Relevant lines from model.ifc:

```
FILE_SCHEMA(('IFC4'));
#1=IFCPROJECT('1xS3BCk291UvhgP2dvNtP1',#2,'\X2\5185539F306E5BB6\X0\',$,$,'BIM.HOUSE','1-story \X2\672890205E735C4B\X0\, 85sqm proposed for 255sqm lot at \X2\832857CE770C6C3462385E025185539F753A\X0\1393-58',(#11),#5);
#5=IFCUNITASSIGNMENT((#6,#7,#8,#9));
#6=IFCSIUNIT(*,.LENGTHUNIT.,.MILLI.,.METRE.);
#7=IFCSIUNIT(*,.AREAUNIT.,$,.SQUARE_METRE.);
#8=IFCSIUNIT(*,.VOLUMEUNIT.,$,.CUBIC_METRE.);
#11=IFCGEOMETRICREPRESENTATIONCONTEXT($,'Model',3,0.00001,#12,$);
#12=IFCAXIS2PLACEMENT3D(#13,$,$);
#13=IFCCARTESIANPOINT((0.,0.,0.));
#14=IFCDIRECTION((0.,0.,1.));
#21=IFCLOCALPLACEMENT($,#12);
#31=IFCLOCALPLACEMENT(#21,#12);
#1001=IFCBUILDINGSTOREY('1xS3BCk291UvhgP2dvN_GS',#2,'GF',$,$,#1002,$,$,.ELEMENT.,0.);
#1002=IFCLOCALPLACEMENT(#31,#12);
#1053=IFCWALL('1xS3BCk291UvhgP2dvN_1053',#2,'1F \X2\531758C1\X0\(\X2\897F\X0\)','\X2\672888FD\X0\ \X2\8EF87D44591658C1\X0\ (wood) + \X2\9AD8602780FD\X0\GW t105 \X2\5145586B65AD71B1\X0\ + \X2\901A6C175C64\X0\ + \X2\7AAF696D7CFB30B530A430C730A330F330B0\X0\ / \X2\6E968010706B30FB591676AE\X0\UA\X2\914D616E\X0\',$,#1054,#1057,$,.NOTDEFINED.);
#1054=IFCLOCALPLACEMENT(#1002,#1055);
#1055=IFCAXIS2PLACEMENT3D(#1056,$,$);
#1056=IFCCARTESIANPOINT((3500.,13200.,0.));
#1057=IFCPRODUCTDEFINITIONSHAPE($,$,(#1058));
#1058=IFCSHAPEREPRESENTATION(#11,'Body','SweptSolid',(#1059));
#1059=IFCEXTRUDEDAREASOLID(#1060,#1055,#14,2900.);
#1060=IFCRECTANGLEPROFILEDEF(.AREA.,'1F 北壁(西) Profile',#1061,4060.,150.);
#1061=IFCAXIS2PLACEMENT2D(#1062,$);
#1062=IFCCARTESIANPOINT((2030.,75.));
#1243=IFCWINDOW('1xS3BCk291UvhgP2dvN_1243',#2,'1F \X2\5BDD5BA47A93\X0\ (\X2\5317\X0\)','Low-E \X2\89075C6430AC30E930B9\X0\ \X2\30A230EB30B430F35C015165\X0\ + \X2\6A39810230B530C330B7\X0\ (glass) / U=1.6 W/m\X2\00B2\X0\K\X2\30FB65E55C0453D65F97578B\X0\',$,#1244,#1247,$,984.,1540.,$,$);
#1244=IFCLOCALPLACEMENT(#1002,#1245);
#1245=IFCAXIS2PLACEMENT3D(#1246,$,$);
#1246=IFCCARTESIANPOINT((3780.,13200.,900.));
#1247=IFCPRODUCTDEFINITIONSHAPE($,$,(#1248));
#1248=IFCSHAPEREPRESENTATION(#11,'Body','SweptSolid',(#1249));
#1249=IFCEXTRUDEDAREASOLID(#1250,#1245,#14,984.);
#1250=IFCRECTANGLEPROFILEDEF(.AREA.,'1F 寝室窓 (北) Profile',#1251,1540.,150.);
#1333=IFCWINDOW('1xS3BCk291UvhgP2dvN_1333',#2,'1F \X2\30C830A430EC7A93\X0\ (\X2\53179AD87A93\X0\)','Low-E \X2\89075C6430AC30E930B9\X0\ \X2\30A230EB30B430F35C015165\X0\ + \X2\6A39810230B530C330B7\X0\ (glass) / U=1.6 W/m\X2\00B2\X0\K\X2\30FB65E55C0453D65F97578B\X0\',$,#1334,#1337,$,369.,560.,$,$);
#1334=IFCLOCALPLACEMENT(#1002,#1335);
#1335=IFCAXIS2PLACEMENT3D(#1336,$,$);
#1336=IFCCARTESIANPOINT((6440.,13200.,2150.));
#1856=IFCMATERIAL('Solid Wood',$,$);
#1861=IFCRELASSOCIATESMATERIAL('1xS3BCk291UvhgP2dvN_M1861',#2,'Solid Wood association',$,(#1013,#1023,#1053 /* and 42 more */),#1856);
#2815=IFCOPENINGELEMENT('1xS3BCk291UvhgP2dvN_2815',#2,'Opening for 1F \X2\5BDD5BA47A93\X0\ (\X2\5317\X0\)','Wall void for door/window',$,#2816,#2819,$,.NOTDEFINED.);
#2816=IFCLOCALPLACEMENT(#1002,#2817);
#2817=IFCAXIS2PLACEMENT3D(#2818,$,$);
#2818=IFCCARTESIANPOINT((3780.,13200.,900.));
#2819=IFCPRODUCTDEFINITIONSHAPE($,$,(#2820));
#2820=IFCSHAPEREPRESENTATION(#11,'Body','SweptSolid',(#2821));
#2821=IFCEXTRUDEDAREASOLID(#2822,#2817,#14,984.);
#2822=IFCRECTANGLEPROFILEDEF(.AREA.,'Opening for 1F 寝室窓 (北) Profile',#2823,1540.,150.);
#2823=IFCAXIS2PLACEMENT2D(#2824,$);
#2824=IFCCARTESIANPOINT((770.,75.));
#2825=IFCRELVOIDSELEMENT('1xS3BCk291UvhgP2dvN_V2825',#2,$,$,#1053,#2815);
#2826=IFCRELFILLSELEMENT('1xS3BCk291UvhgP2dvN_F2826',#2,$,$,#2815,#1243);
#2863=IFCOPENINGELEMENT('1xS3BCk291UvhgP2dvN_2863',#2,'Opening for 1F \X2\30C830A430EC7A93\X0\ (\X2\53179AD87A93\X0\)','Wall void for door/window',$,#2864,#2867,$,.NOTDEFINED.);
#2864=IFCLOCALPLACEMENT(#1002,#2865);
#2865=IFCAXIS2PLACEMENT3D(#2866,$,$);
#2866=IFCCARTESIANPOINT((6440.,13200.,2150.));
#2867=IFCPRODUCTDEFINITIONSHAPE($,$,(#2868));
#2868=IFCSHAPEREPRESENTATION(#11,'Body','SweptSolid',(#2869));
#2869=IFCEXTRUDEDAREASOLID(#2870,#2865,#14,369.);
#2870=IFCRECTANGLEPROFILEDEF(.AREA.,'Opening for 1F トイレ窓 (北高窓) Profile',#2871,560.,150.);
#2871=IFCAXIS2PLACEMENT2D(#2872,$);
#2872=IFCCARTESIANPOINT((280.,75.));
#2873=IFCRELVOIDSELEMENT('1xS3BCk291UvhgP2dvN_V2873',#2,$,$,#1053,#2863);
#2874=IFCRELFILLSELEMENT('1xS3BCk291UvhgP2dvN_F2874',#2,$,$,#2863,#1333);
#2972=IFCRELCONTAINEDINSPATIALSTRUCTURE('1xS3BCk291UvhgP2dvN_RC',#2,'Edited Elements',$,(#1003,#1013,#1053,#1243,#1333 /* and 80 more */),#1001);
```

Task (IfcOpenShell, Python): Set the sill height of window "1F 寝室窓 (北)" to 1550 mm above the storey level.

```python
import numpy as np
import ifcopenshell
import ifcopenshell.api.geometry
import ifcopenshell.geom
import ifcopenshell.util.element
import ifcopenshell.util.placement
import ifcopenshell.util.shape
import ifcopenshell.util.unit

model = ifcopenshell.open("model.ifc")
unit_scale = ifcopenshell.util.unit.calculate_unit_scale(model)

window = model.by_guid("1xS3BCk291UvhgP2dvN_1243")
opening = window.FillsVoids[0].RelatingOpeningElement
storey = ifcopenshell.util.element.get_container(window, ifc_class="IfcBuildingStorey")
level = ifcopenshell.util.placement.get_local_placement(storey.ObjectPlacement)[2, 3]

# The opening's origin need not be at the sill, so measure its lowest point.
shape = ifcopenshell.geom.create_shape(ifcopenshell.geom.settings(), opening)
bottom = ifcopenshell.util.shape.get_shape_bottom_elevation(shape, shape.geometry) / unit_scale
dz = level + 1.55 / unit_scale - bottom

shift = np.array([0.0, 0.0, dz])
# The window is not placed relative to its opening, so move both.
for product in (opening, window):
    matrix = ifcopenshell.util.placement.get_local_placement(product.ObjectPlacement)
    matrix[:3, 3] += shift
    ifcopenshell.api.geometry.edit_object_placement(model, product=product, matrix=matrix, is_si=False)

print(f"moved by {dz * unit_scale:+.3f} m")

model.write("model_edited.ifc")
```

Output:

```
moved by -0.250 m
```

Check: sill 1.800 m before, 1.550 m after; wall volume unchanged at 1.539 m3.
